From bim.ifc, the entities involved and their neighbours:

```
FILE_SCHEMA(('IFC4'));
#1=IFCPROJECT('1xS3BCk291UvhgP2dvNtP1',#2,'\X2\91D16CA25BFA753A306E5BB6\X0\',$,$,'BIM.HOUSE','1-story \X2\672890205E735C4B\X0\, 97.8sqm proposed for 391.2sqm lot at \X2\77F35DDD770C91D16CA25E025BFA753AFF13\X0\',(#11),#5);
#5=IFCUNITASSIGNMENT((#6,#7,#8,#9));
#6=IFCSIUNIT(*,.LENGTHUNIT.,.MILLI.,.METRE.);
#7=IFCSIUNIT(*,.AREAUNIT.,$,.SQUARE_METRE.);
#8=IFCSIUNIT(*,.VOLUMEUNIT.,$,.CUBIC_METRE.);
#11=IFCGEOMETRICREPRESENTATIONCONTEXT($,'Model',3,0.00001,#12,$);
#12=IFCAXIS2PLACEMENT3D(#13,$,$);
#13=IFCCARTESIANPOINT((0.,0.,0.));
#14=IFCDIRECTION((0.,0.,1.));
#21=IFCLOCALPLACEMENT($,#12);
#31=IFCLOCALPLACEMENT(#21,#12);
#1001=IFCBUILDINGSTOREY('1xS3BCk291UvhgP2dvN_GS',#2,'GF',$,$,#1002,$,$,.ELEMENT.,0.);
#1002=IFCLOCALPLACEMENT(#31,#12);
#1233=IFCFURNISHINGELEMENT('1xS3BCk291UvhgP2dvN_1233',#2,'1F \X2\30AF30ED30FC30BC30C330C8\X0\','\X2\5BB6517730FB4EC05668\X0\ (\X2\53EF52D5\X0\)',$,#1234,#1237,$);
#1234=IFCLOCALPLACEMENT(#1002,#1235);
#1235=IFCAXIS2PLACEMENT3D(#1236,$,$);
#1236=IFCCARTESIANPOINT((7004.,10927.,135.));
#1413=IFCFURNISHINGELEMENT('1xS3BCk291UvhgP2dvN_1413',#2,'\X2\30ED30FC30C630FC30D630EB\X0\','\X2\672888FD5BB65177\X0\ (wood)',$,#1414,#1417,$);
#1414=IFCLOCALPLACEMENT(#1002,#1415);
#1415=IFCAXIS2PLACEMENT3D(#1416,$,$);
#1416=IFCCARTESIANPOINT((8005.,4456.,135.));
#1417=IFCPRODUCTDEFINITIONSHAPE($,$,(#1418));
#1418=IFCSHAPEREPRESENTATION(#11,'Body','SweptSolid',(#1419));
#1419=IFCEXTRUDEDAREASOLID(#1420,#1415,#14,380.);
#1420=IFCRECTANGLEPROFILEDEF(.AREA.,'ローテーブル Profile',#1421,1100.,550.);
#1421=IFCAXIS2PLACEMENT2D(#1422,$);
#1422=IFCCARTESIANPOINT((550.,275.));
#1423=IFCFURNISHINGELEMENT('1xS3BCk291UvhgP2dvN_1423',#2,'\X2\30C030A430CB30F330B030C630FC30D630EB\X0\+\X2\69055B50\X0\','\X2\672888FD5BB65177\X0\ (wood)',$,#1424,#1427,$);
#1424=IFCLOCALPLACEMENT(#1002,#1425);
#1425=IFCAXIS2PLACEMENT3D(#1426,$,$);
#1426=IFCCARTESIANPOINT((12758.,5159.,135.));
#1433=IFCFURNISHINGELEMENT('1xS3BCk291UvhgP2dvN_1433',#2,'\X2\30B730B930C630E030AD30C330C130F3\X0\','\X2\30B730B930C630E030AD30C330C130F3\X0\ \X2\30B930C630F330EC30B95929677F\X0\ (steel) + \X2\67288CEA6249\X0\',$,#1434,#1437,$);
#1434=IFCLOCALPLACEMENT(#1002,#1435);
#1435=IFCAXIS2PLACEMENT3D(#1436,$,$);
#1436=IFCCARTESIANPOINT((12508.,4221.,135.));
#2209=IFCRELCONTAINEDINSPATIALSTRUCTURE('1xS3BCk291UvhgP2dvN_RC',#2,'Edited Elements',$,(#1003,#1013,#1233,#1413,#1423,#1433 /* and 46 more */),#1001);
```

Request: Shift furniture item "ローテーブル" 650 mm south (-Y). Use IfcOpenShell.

```python
import ifcopenshell
import ifcopenshell.api.geometry
import ifcopenshell.util.placement

model = ifcopenshell.open("bim.ifc")

item = model.by_guid("1xS3BCk291UvhgP2dvN_1413")
matrix = ifcopenshell.util.placement.get_local_placement(item.ObjectPlacement)
matrix[1, 3] -= 650.0
ifcopenshell.api.geometry.edit_object_placement(model, product=item, matrix=matrix, is_si=False)

print(ifcopenshell.util.placement.get_local_placement(item.ObjectPlacement).round(3) + 0.0)

model.write("bim_updated.ifc")
```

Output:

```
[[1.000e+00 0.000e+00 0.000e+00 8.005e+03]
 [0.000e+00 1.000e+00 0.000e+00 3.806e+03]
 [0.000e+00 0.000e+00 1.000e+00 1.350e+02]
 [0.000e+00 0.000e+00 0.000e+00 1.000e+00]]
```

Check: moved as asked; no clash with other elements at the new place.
